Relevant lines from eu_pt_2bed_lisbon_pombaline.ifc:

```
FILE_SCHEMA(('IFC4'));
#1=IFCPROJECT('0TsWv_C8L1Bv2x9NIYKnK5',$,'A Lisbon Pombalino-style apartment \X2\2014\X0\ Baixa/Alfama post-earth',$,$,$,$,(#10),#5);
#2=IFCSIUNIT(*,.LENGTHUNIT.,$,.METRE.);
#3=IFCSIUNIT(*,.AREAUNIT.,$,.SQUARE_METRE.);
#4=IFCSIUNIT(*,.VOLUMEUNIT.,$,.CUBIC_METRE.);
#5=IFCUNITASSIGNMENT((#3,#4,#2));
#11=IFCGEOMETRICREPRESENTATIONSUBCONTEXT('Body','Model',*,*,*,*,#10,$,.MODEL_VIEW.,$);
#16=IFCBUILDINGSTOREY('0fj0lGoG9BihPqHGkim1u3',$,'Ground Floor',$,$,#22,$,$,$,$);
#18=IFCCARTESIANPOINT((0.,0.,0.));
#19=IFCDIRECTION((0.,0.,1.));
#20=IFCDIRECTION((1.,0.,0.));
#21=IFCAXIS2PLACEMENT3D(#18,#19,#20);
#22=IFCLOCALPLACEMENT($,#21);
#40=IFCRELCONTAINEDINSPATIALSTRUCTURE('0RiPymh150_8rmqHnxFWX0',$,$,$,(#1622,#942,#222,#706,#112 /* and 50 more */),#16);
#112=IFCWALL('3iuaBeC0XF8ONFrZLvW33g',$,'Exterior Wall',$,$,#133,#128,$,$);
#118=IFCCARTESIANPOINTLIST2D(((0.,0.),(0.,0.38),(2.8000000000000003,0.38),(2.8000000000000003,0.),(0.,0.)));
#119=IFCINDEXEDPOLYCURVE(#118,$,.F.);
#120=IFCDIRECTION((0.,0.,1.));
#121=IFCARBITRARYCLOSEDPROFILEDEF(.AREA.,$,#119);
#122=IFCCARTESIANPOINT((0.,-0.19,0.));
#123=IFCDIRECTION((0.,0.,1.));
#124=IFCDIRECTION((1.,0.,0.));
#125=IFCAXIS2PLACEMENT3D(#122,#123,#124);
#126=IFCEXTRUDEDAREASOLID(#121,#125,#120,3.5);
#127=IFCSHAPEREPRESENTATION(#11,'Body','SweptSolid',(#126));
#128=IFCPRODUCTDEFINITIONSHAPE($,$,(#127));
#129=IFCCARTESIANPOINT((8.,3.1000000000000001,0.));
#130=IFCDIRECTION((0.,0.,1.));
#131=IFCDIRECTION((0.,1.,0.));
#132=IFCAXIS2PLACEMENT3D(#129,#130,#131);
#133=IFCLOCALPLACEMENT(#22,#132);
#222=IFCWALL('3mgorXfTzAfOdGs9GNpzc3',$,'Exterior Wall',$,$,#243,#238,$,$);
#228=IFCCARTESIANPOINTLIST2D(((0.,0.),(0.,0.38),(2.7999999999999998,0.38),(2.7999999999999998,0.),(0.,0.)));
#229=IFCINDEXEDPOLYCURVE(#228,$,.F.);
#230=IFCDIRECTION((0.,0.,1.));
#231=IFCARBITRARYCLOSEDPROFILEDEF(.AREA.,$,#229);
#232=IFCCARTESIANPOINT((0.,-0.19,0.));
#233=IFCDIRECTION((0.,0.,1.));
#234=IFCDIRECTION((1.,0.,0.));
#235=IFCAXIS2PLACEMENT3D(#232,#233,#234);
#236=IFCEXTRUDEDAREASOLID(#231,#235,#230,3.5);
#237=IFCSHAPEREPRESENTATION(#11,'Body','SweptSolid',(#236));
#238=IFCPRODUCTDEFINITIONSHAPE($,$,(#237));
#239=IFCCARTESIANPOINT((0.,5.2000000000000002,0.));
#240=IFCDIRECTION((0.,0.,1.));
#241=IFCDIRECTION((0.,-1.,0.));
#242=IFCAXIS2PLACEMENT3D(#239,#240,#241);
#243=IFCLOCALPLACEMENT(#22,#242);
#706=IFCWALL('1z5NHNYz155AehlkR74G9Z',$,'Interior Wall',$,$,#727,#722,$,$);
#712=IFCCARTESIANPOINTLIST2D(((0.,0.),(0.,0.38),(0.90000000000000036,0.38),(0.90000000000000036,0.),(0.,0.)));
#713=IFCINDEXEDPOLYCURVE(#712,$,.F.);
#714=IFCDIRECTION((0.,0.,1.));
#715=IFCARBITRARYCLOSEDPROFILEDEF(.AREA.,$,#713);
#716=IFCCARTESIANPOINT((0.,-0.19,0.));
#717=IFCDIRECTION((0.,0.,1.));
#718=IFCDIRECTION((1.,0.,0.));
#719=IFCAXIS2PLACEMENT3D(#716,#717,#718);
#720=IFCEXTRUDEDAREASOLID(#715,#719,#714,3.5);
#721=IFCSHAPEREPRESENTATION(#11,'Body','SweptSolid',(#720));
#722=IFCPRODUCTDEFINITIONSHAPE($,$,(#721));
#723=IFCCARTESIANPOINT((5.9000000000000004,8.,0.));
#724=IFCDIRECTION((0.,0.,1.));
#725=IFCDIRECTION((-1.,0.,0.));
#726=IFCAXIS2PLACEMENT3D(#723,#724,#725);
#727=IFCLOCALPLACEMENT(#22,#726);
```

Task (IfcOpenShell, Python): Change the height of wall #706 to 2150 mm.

```python
import ifcopenshell
import ifcopenshell.geom
import ifcopenshell.util.representation
import ifcopenshell.util.shape

model = ifcopenshell.open("eu_pt_2bed_lisbon_pombaline.ifc")
settings = ifcopenshell.geom.settings()


def volume(element):
    """Net volume in cubic metres, openings subtracted."""
    shape = ifcopenshell.geom.create_shape(settings, element)
    return ifcopenshell.util.shape.get_volume(shape.geometry)


wall = model.by_guid("1z5NHNYz155AehlkR74G9Z")
before = volume(wall)

body = ifcopenshell.util.representation.get_representation(wall, "Model", "Body")
solid = body.Items[0]
old_height = solid.Depth
solid.Depth = 2.15
after = volume(wall)

print(f"height {old_height:g} -> {solid.Depth:g}, volume {before:.3f} -> {after:.3f} m3")

model.write("eu_pt_2bed_lisbon_pombaline_edited.ifc")
```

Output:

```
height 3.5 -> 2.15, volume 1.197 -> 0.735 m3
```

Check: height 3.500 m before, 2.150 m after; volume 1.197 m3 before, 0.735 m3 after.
